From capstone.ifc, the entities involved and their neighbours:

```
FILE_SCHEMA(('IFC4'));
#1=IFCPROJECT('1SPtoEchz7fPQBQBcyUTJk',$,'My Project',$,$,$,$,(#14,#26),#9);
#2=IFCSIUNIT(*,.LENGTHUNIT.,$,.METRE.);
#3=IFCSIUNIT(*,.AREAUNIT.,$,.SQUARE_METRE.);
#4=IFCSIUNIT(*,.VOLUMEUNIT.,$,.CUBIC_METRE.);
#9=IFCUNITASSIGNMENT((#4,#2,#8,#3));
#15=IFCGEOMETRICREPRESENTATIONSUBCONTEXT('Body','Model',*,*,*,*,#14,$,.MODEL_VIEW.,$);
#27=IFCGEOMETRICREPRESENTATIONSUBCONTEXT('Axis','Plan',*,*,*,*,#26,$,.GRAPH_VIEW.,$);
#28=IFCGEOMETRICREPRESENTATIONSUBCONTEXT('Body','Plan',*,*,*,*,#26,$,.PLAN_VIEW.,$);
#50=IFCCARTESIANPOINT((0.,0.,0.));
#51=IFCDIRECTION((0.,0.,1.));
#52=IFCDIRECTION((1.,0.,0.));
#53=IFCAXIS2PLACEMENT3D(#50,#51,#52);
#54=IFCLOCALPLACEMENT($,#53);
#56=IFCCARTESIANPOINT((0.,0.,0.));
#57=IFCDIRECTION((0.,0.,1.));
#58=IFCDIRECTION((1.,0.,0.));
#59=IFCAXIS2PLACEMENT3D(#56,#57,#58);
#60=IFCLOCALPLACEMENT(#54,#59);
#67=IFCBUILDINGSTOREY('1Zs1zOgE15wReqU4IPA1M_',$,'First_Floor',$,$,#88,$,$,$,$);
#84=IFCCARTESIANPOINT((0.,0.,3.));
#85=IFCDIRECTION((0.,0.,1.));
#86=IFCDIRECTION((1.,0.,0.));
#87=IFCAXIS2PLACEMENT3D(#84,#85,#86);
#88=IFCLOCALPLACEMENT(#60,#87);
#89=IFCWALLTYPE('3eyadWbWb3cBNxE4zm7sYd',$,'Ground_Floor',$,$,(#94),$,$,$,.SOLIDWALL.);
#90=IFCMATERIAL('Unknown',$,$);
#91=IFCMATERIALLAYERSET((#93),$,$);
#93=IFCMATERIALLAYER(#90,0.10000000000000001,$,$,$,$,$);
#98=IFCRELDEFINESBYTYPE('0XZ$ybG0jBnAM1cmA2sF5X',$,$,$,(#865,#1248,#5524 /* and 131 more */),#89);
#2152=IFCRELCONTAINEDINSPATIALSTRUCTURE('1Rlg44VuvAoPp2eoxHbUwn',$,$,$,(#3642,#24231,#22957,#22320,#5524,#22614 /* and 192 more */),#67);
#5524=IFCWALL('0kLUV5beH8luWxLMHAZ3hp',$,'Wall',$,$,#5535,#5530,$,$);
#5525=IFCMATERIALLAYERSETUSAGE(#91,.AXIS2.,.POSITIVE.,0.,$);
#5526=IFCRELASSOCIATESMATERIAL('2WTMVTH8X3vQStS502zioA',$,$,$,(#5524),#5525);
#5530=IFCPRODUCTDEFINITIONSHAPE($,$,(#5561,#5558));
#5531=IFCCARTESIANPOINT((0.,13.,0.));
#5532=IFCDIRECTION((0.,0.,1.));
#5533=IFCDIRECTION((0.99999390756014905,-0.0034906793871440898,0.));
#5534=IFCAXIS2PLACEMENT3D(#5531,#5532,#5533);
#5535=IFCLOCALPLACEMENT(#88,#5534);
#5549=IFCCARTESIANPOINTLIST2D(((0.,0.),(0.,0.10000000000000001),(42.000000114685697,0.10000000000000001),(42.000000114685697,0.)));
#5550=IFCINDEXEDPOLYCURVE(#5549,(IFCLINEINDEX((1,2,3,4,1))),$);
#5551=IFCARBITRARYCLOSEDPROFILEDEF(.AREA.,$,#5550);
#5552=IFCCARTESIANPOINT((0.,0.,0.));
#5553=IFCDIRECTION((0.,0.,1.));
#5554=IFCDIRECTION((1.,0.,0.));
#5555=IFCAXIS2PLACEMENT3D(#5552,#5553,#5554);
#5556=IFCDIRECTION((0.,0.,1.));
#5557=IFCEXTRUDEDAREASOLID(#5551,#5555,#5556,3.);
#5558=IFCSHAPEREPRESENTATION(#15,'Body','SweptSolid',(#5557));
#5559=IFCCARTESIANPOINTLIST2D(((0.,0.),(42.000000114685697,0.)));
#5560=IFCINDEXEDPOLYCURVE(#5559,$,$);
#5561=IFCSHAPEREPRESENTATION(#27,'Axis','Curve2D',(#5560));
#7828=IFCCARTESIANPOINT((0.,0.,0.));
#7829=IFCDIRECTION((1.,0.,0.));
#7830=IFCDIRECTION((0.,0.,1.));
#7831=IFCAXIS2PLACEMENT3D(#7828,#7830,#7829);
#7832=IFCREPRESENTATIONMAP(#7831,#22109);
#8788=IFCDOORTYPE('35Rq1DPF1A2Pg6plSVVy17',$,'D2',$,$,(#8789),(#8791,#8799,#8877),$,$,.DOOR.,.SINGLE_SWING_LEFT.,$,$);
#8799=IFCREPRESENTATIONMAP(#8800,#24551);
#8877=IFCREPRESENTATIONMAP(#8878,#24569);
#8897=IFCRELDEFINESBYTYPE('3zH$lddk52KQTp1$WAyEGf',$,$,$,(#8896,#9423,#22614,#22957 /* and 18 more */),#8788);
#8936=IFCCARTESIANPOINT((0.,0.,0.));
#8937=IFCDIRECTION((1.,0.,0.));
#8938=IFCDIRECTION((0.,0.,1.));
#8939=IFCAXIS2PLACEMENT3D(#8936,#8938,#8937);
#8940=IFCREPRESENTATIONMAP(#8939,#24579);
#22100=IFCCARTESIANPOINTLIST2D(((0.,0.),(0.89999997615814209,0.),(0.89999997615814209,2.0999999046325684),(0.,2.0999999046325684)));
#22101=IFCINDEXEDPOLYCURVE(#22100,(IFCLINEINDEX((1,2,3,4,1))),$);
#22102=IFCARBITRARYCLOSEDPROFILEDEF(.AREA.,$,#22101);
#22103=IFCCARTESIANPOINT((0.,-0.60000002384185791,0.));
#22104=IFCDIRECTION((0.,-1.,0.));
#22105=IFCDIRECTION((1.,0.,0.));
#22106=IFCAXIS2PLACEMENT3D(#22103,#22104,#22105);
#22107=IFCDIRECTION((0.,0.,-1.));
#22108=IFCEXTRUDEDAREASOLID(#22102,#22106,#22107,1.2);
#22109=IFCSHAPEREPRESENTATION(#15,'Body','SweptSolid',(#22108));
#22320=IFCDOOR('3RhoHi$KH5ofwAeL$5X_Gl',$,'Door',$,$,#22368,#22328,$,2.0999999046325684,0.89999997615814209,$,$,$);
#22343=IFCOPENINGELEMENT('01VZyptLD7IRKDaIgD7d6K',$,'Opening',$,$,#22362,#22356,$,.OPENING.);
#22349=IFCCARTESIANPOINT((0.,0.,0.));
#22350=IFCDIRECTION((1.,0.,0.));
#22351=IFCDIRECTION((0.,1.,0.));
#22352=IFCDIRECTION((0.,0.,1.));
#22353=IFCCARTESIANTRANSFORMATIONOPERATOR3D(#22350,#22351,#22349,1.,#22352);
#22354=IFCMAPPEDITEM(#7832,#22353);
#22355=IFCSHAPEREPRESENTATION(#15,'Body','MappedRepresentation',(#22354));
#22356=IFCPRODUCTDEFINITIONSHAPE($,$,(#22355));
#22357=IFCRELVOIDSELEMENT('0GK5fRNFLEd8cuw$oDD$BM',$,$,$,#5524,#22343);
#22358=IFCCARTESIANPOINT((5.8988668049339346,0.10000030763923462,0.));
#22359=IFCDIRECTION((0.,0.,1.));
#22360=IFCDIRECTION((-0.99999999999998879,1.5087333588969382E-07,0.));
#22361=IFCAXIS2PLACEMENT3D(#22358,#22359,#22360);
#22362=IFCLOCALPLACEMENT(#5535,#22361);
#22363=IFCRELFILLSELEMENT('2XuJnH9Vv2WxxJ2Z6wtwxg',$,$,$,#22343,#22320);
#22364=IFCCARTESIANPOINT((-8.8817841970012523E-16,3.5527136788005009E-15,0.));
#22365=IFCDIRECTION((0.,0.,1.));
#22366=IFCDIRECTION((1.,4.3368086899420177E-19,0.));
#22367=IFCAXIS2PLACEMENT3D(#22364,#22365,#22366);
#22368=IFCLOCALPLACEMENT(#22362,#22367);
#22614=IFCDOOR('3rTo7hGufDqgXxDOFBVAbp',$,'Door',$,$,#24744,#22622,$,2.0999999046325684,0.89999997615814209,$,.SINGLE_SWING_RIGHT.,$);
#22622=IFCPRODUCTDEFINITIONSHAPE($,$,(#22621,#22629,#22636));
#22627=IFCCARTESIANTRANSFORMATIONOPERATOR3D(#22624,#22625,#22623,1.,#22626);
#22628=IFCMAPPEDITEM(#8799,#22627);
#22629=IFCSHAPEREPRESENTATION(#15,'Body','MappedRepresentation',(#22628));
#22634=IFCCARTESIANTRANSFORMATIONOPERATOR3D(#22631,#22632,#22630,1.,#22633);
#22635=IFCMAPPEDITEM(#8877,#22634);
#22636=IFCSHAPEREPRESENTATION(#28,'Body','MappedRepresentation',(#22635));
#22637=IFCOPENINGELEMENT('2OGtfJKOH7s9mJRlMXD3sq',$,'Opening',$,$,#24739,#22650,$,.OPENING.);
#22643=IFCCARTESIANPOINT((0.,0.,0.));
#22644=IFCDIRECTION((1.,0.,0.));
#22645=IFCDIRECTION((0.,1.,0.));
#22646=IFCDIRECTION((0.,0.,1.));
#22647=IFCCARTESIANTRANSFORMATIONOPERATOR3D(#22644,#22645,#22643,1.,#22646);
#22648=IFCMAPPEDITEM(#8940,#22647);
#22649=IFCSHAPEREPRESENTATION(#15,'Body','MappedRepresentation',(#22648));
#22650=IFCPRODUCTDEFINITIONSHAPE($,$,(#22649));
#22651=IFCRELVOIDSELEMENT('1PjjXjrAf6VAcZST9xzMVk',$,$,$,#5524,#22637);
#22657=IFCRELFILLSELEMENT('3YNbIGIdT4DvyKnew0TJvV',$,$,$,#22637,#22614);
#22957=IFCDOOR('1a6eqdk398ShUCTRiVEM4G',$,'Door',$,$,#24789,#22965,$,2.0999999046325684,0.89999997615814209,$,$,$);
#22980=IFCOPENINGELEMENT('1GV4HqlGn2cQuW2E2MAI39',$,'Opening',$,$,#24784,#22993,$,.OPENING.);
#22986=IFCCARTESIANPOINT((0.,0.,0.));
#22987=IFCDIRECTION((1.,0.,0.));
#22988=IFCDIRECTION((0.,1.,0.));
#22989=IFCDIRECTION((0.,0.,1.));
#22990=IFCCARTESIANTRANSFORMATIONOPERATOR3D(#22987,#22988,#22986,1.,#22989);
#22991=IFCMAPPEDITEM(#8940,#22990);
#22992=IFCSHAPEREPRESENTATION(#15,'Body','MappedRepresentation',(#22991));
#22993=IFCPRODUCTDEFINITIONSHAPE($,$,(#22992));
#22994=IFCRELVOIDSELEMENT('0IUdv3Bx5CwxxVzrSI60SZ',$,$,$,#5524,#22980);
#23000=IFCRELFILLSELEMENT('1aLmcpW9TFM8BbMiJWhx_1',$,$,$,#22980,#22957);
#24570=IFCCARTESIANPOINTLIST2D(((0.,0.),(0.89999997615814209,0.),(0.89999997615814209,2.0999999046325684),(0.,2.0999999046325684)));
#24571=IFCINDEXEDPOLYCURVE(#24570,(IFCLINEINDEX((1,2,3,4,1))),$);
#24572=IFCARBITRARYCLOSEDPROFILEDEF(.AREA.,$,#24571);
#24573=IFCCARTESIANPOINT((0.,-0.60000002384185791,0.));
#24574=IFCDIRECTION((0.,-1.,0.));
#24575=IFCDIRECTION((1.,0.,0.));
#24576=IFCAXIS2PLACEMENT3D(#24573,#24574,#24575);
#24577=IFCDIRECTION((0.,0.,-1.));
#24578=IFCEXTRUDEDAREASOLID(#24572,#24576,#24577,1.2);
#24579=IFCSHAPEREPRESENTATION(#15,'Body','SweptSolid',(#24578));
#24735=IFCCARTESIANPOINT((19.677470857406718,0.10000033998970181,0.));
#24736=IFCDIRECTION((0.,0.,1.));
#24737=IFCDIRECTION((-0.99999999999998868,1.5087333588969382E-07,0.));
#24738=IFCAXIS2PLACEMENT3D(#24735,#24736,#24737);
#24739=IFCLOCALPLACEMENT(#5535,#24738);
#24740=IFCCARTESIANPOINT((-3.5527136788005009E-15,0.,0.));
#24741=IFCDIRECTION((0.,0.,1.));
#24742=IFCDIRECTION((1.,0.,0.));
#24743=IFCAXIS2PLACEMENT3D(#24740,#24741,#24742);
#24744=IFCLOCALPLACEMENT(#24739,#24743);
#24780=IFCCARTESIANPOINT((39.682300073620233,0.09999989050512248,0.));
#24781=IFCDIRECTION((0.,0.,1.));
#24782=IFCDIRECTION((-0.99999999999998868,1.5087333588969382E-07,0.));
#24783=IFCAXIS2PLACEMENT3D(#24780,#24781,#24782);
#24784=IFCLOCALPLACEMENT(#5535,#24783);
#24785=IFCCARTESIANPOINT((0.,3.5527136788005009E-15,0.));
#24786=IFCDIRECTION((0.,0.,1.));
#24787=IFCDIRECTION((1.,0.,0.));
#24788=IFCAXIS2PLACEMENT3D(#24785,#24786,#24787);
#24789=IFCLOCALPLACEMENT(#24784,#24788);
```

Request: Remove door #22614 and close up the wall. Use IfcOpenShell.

```python
import ifcopenshell
import ifcopenshell.api.feature
import ifcopenshell.api.root
import ifcopenshell.geom
import ifcopenshell.util.shape

model = ifcopenshell.open("capstone.ifc")
settings = ifcopenshell.geom.settings()


def volume(element):
    """Net volume in cubic metres, openings subtracted."""
    shape = ifcopenshell.geom.create_shape(settings, element)
    return ifcopenshell.util.shape.get_volume(shape.geometry)


door = model.by_guid("3rTo7hGufDqgXxDOFBVAbp")
opening = door.FillsVoids[0].RelatingOpeningElement
wall = opening.VoidsElements[0].RelatingBuildingElement
before = volume(wall)

ifcopenshell.api.root.remove_product(model, product=door)
ifcopenshell.api.feature.remove_feature(model, feature=opening)

after = volume(wall)

print(f"wall volume {before:.3f} -> {after:.3f} m3")

model.write("capstone-out.ifc")
```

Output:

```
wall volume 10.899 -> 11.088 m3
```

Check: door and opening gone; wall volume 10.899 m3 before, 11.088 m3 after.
